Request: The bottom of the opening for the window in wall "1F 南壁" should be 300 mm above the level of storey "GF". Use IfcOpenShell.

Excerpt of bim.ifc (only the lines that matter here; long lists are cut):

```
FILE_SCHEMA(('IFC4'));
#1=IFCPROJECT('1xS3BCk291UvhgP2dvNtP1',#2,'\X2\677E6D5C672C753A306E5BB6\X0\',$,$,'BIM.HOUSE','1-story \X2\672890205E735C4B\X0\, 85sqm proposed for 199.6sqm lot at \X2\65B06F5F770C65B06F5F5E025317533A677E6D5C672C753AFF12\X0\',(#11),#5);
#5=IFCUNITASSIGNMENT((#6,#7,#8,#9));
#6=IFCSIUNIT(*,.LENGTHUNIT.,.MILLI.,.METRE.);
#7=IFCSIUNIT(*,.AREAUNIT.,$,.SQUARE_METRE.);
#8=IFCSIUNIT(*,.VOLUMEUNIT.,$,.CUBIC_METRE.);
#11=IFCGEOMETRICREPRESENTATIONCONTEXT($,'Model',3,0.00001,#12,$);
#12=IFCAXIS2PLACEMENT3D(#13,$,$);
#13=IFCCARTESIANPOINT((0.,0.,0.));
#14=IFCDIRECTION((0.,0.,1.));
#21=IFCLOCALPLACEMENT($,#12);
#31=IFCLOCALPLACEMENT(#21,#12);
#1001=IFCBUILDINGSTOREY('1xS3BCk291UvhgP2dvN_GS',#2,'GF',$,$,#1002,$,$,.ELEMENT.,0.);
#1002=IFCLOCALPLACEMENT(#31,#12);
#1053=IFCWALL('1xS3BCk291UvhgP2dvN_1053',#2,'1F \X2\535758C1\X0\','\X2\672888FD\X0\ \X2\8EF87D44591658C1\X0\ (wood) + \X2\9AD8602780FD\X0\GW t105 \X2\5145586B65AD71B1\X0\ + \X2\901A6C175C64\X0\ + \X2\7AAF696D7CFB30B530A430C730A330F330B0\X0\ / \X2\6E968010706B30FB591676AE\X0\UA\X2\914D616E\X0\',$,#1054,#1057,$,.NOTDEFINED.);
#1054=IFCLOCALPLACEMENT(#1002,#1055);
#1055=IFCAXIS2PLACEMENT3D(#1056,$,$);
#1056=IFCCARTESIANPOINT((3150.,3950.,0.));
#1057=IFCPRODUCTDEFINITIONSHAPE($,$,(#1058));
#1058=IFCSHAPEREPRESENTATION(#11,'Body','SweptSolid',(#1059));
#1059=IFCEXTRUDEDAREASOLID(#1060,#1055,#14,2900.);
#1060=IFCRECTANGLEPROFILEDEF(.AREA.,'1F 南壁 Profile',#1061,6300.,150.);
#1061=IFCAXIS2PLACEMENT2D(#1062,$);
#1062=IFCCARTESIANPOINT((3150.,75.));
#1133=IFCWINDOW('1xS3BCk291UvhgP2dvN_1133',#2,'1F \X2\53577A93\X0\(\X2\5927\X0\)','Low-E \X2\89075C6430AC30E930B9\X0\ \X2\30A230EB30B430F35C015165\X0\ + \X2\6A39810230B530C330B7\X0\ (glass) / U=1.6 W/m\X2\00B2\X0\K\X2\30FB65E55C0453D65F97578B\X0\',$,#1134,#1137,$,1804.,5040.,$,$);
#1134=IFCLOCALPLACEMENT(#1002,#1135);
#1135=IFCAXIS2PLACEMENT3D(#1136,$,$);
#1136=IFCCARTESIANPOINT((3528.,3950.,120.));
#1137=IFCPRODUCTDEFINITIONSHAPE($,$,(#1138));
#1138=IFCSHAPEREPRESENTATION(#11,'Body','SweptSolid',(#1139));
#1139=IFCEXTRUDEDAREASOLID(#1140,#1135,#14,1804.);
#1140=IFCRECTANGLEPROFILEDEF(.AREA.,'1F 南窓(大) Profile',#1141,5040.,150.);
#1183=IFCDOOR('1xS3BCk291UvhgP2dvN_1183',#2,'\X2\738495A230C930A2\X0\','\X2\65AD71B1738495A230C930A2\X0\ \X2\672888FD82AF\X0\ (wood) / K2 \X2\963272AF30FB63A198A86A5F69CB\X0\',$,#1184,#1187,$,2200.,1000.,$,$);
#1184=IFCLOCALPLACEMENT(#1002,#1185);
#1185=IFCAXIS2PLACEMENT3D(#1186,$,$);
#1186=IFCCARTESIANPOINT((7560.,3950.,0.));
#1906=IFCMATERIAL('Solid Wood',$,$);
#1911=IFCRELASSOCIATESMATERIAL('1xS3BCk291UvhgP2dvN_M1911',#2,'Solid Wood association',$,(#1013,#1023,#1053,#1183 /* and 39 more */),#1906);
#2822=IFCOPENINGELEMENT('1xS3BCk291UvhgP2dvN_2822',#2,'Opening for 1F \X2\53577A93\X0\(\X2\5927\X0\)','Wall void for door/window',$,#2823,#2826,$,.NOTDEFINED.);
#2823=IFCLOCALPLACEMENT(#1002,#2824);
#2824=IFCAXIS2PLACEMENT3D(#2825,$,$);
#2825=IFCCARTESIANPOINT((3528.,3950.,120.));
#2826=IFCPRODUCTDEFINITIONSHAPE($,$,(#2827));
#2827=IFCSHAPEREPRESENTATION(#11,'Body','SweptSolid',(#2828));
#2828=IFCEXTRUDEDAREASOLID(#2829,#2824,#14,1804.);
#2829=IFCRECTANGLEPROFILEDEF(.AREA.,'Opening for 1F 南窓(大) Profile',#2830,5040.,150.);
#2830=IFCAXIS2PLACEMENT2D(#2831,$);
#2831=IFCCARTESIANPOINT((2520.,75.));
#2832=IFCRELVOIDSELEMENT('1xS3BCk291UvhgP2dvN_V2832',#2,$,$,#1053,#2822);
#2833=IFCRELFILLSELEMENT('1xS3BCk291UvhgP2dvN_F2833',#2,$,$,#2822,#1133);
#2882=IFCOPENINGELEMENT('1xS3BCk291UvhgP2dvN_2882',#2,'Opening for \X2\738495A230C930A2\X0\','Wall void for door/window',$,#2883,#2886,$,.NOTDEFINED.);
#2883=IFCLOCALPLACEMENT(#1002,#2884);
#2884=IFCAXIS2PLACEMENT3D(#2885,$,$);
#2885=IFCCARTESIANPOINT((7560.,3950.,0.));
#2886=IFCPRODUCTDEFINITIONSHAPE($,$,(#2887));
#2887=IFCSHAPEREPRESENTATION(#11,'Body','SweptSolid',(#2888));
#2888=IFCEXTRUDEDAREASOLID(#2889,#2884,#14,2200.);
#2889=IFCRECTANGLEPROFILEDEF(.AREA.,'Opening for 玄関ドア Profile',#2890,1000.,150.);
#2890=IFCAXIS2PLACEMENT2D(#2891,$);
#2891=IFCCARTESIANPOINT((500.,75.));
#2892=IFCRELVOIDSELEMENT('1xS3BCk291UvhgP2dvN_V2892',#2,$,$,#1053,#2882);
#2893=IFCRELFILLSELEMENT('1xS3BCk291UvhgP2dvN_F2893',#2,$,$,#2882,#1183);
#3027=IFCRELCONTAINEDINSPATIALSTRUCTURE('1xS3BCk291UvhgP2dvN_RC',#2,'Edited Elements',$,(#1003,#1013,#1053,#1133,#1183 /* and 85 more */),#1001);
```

```python
import numpy as np
import ifcopenshell
import ifcopenshell.api.geometry
import ifcopenshell.geom
import ifcopenshell.util.element
import ifcopenshell.util.placement
import ifcopenshell.util.shape
import ifcopenshell.util.unit

model = ifcopenshell.open("bim.ifc")
unit_scale = ifcopenshell.util.unit.calculate_unit_scale(model)

window = model.by_guid("1xS3BCk291UvhgP2dvN_1133")
opening = window.FillsVoids[0].RelatingOpeningElement
storey = ifcopenshell.util.element.get_container(window, ifc_class="IfcBuildingStorey")
level = ifcopenshell.util.placement.get_local_placement(storey.ObjectPlacement)[2, 3]

# The opening's origin need not be at the sill, so measure its lowest point.
shape = ifcopenshell.geom.create_shape(ifcopenshell.geom.settings(), opening)
bottom = ifcopenshell.util.shape.get_shape_bottom_elevation(shape, shape.geometry) / unit_scale
dz = level + 0.3 / unit_scale - bottom

shift = np.array([0.0, 0.0, dz])
# The window is not placed relative to its opening, so move both.
for product in (opening, window):
    matrix = ifcopenshell.util.placement.get_local_placement(product.ObjectPlacement)
    matrix[:3, 3] += shift
    ifcopenshell.api.geometry.edit_object_placement(model, product=product, matrix=matrix, is_si=False)

print(f"moved by {dz * unit_scale:+.3f} m")

model.write("bim-out.ifc")
```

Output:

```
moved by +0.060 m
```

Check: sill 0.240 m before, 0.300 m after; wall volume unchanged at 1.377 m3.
